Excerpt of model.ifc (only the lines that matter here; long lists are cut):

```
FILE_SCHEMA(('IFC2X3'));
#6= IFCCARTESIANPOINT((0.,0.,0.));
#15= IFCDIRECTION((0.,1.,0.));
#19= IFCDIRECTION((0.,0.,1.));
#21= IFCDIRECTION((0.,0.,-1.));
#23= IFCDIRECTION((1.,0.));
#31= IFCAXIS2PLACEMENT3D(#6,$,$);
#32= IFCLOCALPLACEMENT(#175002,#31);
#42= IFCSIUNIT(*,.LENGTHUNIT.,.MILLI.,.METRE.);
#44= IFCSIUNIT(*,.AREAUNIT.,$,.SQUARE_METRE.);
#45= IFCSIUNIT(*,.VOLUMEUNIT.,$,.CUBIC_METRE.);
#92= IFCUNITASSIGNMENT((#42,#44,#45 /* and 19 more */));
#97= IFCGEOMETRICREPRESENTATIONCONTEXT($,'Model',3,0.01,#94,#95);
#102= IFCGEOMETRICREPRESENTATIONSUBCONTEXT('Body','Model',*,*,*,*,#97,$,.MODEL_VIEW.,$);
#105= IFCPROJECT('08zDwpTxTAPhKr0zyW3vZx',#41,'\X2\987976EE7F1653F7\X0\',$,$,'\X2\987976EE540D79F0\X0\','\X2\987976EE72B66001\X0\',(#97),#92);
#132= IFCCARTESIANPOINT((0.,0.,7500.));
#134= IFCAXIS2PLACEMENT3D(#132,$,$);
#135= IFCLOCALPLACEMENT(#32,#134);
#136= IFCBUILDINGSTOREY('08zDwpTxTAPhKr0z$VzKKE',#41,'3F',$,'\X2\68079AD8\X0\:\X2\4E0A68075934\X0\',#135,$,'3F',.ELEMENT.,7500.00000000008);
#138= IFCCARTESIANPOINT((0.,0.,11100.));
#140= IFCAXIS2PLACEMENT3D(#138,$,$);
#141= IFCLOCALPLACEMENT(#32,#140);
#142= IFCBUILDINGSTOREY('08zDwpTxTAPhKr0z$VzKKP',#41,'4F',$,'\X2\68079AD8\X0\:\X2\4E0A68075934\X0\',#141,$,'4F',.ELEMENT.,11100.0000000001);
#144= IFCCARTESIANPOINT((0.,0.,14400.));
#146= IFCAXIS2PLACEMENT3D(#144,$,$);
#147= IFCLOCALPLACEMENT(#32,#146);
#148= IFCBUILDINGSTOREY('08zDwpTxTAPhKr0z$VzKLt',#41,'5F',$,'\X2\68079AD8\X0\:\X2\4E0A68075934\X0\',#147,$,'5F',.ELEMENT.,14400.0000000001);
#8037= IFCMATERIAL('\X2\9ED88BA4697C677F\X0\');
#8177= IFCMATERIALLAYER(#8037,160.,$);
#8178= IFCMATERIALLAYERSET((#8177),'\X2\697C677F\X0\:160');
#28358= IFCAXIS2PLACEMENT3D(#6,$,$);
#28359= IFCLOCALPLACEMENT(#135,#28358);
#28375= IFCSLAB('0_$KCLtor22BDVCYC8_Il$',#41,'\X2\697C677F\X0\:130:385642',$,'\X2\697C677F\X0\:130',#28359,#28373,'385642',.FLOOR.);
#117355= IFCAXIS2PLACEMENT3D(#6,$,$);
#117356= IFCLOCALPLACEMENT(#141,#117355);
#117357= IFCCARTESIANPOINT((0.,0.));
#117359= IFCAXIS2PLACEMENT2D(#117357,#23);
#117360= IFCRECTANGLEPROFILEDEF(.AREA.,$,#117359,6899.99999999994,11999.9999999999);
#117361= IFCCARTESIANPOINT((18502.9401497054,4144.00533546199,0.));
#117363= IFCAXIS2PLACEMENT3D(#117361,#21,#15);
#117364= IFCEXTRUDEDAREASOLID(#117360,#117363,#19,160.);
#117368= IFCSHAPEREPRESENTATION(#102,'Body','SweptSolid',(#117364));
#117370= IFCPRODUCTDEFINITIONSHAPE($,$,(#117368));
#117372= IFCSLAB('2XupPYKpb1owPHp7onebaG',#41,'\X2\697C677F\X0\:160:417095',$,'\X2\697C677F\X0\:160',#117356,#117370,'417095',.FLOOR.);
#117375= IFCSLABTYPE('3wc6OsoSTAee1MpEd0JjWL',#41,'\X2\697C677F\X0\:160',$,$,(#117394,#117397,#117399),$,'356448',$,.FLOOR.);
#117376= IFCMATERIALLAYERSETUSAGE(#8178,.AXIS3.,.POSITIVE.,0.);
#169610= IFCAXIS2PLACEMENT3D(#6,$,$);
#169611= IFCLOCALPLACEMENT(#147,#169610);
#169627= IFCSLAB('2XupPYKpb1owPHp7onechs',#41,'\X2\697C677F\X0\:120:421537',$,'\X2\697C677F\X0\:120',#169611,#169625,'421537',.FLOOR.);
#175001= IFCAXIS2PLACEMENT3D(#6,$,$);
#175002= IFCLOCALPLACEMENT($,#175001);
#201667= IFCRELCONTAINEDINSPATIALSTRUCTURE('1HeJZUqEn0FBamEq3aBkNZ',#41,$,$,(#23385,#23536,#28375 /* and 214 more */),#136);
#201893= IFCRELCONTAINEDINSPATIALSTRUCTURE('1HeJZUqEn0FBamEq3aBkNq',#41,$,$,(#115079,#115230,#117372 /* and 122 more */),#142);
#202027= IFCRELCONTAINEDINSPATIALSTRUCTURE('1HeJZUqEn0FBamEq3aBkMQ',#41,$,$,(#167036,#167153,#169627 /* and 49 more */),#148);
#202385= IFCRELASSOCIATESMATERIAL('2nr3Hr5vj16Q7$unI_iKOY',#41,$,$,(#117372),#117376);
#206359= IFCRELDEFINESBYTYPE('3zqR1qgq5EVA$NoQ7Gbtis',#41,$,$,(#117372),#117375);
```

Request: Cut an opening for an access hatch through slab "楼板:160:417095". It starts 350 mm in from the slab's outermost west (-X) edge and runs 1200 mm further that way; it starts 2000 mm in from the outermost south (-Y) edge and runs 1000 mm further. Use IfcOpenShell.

```python
import numpy as np
import ifcopenshell
import ifcopenshell.api.feature
import ifcopenshell.api.geometry
import ifcopenshell.api.root
import ifcopenshell.geom
import ifcopenshell.util.placement
import ifcopenshell.util.representation
import ifcopenshell.util.shape
import ifcopenshell.util.unit

model = ifcopenshell.open("model.ifc")
unit_scale = ifcopenshell.util.unit.calculate_unit_scale(model)
settings = ifcopenshell.geom.settings()


def volume(element):
    """Net volume in cubic metres, openings subtracted."""
    shape = ifcopenshell.geom.create_shape(settings, element)
    return ifcopenshell.util.shape.get_volume(shape.geometry)


slab = model.by_guid("2XupPYKpb1owPHp7onebaG")
before = volume(slab)

# Extent in the slab's own axes, in metres. The edges named are its -X and -Y sides.
slab_shape = ifcopenshell.geom.create_shape(settings, slab)
vertices = ifcopenshell.util.shape.get_vertices(slab_shape.geometry)
x_min, y_min, bottom = vertices.min(axis=0)
top = vertices[:, 2].max()

opening = ifcopenshell.api.root.create_entity(model, ifc_class="IfcOpeningElement", name="Access hatch opening")
context = ifcopenshell.util.representation.get_context(model, "Model", "Body", "MODEL_VIEW")
width, depth = 1.2, 1
outline = [(0.0, 0.0), (width, 0.0), (width, depth), (0.0, depth), (0.0, 0.0)]
# Overshoot both faces by 50 mm so the cut is clean.
shape = ifcopenshell.api.geometry.add_slab_representation(
    model, context=context, depth=top - bottom + 0.1, polyline=outline
)
ifcopenshell.api.geometry.assign_representation(model, product=opening, representation=shape)

matrix = ifcopenshell.util.placement.get_local_placement(slab.ObjectPlacement)
matrix[:, 3] = matrix @ np.append(np.array([x_min + 0.35, y_min + 2, bottom - 0.05]) / unit_scale, 1.0)
ifcopenshell.api.geometry.edit_object_placement(model, product=opening, matrix=matrix, is_si=False)
ifcopenshell.api.feature.add_feature(model, feature=opening, element=slab)

after = volume(slab)

print(f"slab volume {before:.3f} -> {after:.3f} m3")

model.write("model-out.ifc")
```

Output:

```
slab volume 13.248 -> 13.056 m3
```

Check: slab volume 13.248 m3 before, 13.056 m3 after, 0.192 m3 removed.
